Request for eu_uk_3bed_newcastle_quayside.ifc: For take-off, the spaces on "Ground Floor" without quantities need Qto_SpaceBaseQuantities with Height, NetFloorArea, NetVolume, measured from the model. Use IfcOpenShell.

First a look at what the model holds.

```python
import ifcopenshell
import ifcopenshell.util.element
import ifcopenshell.util.unit

model = ifcopenshell.open("eu_uk_3bed_newcastle_quayside.ifc")
print(model.schema)
for unit_type in ("LENGTHUNIT", "AREAUNIT", "VOLUMEUNIT"):
    print(unit_type, ifcopenshell.util.unit.calculate_unit_scale(model, unit_type))
storey = next(s for s in model.by_type("IfcBuildingStorey") if s.Name == "Ground Floor")
spaces = [e for e in ifcopenshell.util.element.get_decomposition(storey) if e.is_a("IfcSpace")]
for e in sorted(spaces, key=lambda e: e.id()):
    print(e.id(), e.is_a(), e.Name, list(ifcopenshell.util.element.get_psets(e, qtos_only=True)), sep=" | ")
```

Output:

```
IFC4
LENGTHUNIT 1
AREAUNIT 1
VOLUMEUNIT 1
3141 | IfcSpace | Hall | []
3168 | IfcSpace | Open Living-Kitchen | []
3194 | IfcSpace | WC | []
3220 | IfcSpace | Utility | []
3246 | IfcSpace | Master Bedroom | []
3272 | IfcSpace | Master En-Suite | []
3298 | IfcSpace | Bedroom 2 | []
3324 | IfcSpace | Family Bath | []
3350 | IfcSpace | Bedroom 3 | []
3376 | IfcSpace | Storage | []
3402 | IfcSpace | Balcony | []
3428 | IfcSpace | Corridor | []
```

```python
import ifcopenshell
import ifcopenshell.api.pset
import ifcopenshell.geom
import ifcopenshell.util.element
import ifcopenshell.util.shape
import ifcopenshell.util.unit

model = ifcopenshell.open("eu_uk_3bed_newcastle_quayside.ifc")
unit_scale = ifcopenshell.util.unit.calculate_unit_scale(model)
area_scale = ifcopenshell.util.unit.calculate_unit_scale(model, "AREAUNIT")
volume_scale = ifcopenshell.util.unit.calculate_unit_scale(model, "VOLUMEUNIT")
settings = ifcopenshell.geom.settings()

storey = next(s for s in model.by_type("IfcBuildingStorey") if s.Name == "Ground Floor")
spaces = [e for e in ifcopenshell.util.element.get_decomposition(storey) if e.is_a("IfcSpace")]

for e in sorted(spaces, key=lambda e: e.id()):
    if ifcopenshell.util.element.get_psets(e, qtos_only=True, should_inherit=False):
        continue
    # Geometry comes back in metres, in the element's own axes.
    shape = ifcopenshell.geom.create_shape(settings, e)
    values = {
        "Height": ifcopenshell.util.shape.get_z(shape.geometry) / unit_scale,
        "NetFloorArea": ifcopenshell.util.shape.get_footprint_area(shape.geometry) / area_scale,
        "NetVolume": ifcopenshell.util.shape.get_volume(shape.geometry) / volume_scale,
    }
    qto = ifcopenshell.api.pset.add_qto(model, product=e, name="Qto_SpaceBaseQuantities")
    ifcopenshell.api.pset.edit_qto(model, qto=qto, properties=values)
    print(e.id(), {k: round(v, 3) for k, v in values.items()})

model.write("eu_uk_3bed_newcastle_quayside_edited.ifc")
```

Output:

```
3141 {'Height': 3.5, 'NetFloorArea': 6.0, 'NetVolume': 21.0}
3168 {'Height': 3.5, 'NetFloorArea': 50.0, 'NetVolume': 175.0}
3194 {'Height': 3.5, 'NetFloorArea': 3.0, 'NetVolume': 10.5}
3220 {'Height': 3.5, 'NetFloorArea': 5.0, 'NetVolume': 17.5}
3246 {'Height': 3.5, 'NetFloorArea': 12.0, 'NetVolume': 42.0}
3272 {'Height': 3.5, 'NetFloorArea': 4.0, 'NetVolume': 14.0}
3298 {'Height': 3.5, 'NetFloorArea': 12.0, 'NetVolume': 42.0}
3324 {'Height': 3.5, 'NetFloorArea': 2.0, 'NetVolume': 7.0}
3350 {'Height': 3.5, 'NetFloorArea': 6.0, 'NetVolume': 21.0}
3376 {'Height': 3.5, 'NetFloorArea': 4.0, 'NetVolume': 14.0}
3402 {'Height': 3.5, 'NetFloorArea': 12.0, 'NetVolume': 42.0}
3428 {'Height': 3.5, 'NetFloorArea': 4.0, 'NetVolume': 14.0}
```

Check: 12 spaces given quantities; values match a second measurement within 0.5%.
